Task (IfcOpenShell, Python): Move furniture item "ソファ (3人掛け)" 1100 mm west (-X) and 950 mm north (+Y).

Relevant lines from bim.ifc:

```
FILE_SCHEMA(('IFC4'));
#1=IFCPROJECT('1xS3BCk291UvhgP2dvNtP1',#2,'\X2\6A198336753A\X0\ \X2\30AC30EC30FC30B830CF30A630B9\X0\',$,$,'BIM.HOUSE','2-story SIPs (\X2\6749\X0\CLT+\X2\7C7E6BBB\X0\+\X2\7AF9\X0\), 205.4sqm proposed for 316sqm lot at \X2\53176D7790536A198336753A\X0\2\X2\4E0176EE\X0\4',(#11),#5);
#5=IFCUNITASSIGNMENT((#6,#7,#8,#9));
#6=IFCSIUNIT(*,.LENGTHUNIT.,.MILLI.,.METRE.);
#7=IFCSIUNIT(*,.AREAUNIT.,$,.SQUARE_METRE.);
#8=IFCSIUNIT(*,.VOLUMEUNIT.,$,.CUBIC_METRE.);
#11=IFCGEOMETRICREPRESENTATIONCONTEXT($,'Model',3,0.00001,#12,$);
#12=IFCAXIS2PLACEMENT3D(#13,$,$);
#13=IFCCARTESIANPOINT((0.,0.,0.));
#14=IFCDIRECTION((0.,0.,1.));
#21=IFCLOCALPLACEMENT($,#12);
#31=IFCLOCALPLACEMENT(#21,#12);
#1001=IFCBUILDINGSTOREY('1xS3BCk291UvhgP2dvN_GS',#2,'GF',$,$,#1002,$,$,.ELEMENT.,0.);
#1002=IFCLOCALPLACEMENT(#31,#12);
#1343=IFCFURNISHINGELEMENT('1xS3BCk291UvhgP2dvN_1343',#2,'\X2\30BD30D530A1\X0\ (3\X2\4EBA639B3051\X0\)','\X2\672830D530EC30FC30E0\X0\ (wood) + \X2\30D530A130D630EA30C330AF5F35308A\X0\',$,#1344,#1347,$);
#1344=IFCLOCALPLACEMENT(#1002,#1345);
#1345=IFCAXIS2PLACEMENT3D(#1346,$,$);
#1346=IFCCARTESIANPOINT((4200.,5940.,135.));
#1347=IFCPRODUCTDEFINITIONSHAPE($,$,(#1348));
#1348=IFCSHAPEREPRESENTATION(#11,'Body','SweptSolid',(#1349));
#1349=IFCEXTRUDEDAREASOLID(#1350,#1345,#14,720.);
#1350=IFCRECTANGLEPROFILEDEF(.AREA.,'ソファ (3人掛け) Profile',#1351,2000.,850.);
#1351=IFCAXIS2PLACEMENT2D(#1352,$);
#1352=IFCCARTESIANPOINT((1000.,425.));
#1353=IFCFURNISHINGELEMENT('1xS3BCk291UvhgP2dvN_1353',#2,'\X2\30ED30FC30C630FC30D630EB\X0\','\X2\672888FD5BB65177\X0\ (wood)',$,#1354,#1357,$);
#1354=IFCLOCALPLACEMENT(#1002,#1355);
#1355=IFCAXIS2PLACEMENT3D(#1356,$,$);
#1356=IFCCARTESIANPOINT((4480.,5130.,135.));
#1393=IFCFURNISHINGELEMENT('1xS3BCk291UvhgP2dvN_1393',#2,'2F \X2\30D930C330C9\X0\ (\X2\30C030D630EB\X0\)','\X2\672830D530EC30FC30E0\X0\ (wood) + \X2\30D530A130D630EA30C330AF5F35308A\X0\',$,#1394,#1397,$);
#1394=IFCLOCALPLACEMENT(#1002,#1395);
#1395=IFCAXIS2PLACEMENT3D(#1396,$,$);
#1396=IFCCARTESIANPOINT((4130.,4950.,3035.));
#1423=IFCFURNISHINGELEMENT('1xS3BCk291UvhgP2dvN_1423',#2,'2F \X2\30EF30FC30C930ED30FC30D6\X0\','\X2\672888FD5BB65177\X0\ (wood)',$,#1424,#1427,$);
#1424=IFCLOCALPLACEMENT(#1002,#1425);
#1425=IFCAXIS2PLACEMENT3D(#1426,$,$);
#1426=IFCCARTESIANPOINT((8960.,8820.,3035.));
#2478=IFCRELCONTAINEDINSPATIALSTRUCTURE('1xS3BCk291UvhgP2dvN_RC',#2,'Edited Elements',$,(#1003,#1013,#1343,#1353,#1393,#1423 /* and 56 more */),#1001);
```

```python
import ifcopenshell
import ifcopenshell.api.geometry
import ifcopenshell.util.placement

model = ifcopenshell.open("bim.ifc")

item = model.by_guid("1xS3BCk291UvhgP2dvN_1343")
matrix = ifcopenshell.util.placement.get_local_placement(item.ObjectPlacement)
matrix[0, 3] -= 1100.0
matrix[1, 3] += 950.0
ifcopenshell.api.geometry.edit_object_placement(model, product=item, matrix=matrix, is_si=False)

print(ifcopenshell.util.placement.get_local_placement(item.ObjectPlacement).round(3) + 0.0)

model.write("bim_updated.ifc")
```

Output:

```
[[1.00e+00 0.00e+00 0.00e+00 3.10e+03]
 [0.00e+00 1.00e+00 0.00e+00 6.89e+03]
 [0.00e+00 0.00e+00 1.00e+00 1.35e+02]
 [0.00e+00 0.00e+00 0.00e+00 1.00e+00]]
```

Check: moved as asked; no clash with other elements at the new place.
